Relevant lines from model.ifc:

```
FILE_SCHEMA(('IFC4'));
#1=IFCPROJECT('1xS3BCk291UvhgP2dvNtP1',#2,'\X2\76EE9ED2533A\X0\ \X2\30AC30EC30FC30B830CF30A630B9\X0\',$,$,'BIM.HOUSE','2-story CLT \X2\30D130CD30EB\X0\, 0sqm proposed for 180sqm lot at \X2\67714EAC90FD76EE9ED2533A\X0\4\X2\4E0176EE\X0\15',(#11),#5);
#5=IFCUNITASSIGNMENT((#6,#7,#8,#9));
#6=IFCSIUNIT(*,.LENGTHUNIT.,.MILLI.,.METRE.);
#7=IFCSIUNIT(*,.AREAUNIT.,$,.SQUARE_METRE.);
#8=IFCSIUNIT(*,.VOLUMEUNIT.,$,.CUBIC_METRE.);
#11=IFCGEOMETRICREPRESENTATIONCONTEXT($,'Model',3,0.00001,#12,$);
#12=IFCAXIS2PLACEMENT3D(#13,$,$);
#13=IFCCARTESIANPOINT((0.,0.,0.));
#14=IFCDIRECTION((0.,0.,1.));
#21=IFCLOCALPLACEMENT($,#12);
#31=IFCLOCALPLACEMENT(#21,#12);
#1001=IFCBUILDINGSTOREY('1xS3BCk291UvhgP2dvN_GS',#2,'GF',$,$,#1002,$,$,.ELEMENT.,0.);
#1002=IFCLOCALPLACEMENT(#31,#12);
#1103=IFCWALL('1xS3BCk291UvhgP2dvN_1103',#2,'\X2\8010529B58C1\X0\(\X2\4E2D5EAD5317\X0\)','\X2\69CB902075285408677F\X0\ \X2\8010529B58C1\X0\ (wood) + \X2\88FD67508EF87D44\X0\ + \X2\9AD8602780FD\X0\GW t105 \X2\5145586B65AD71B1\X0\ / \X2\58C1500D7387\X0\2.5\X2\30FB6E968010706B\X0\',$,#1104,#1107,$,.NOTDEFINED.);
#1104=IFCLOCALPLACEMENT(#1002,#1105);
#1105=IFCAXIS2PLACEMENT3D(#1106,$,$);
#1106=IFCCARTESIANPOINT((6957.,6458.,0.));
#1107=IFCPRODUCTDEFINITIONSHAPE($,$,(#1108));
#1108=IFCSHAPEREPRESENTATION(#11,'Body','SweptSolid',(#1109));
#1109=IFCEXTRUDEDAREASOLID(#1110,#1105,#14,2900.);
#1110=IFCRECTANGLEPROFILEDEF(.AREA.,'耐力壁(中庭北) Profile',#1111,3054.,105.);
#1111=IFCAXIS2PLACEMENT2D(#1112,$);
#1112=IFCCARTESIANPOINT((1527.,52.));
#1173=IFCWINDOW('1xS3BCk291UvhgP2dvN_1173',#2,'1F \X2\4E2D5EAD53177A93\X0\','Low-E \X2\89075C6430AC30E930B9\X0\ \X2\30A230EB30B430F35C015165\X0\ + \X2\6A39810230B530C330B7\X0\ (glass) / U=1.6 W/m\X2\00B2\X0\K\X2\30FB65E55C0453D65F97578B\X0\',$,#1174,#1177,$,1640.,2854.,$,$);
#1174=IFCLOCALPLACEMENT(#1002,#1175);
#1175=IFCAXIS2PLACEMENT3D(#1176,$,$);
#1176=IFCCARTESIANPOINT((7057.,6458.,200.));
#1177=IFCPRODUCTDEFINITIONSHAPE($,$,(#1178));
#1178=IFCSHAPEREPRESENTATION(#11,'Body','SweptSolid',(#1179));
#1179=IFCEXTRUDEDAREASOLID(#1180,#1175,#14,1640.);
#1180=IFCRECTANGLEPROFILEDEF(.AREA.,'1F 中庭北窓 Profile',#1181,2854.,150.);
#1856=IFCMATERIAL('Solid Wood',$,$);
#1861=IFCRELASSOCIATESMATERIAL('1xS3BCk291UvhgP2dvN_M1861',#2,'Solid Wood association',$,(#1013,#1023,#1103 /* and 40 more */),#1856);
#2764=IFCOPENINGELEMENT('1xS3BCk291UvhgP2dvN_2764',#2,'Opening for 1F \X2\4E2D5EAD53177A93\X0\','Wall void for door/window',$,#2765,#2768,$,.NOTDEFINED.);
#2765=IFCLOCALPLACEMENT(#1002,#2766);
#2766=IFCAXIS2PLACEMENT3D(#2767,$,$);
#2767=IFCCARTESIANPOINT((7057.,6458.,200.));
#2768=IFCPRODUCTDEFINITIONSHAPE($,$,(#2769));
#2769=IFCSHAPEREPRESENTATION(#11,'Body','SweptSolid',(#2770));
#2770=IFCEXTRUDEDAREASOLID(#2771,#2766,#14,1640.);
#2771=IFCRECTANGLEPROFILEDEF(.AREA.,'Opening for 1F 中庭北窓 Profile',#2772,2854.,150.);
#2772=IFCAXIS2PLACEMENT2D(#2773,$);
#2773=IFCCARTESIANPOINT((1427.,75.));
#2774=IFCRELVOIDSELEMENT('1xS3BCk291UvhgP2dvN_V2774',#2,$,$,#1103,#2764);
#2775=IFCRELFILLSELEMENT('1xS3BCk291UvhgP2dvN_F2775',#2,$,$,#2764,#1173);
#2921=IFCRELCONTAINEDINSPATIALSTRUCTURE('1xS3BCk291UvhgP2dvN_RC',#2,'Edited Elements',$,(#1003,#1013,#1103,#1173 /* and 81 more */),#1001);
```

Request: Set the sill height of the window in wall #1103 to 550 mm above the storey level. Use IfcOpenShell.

```python
import numpy as np
import ifcopenshell
import ifcopenshell.api.geometry
import ifcopenshell.geom
import ifcopenshell.util.element
import ifcopenshell.util.placement
import ifcopenshell.util.shape
import ifcopenshell.util.unit

model = ifcopenshell.open("model.ifc")
unit_scale = ifcopenshell.util.unit.calculate_unit_scale(model)

window = model.by_guid("1xS3BCk291UvhgP2dvN_1173")
opening = window.FillsVoids[0].RelatingOpeningElement
storey = ifcopenshell.util.element.get_container(window, ifc_class="IfcBuildingStorey")
level = ifcopenshell.util.placement.get_local_placement(storey.ObjectPlacement)[2, 3]

# The opening's origin need not be at the sill, so measure its lowest point.
shape = ifcopenshell.geom.create_shape(ifcopenshell.geom.settings(), opening)
bottom = ifcopenshell.util.shape.get_shape_bottom_elevation(shape, shape.geometry) / unit_scale
dz = level + 550.0 - bottom

shift = np.array([0.0, 0.0, dz])
# The window is not placed relative to its opening, so move both.
for product in (opening, window):
    matrix = ifcopenshell.util.placement.get_local_placement(product.ObjectPlacement)
    matrix[:3, 3] += shift
    ifcopenshell.api.geometry.edit_object_placement(model, product=product, matrix=matrix, is_si=False)

print(f"moved by {dz * unit_scale:+.3f} m")

model.write("model_rev.ifc")
```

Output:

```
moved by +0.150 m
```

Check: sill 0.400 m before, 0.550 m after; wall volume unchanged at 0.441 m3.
